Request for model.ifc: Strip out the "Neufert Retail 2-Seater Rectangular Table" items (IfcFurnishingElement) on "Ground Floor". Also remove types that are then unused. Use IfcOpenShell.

First a look at what the model holds.

```python
import ifcopenshell
import ifcopenshell.util.element

model = ifcopenshell.open("model.ifc")
print(model.schema)
storey = next(s for s in model.by_type("IfcBuildingStorey") if s.Name == "Ground Floor")
furniture = [e for e in ifcopenshell.util.element.get_decomposition(storey) if e.is_a("IfcFurnishingElement")]
seen = {}
for e in furniture:
    element_type = ifcopenshell.util.element.get_type(e)
    name = element_type.Name if element_type not in (None, e) else None
    seen[name] = seen.get(name, 0) + 1
for name, count in sorted(seen.items(), key=str):
    print(count, "x", name)
```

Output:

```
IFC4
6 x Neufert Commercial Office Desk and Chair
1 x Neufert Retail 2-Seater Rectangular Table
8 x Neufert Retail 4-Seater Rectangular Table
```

```python
import ifcopenshell
import ifcopenshell.api.root
import ifcopenshell.util.element

model = ifcopenshell.open("model.ifc")

storey = next(s for s in model.by_type("IfcBuildingStorey") if s.Name == "Ground Floor")
furniture = [e for e in ifcopenshell.util.element.get_decomposition(storey) if e.is_a("IfcFurnishingElement")]
targets = [e for e in furniture if (t := ifcopenshell.util.element.get_type(e)) not in (None, e) and t.Name == "Neufert Retail 2-Seater Rectangular Table"]
types = {ifcopenshell.util.element.get_type(e) for e in targets} - {None, *targets}

for e in targets:
    ifcopenshell.api.root.remove_product(model, product=e)
print(len(targets), "removed")

unused = [t for t in types if not ifcopenshell.util.element.get_types(t)]
for t in unused:
    ifcopenshell.api.root.remove_product(model, product=t)
print(len(unused), "unused types removed")

model.write("model_updated.ifc")
```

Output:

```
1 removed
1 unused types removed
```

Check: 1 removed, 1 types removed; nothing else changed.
